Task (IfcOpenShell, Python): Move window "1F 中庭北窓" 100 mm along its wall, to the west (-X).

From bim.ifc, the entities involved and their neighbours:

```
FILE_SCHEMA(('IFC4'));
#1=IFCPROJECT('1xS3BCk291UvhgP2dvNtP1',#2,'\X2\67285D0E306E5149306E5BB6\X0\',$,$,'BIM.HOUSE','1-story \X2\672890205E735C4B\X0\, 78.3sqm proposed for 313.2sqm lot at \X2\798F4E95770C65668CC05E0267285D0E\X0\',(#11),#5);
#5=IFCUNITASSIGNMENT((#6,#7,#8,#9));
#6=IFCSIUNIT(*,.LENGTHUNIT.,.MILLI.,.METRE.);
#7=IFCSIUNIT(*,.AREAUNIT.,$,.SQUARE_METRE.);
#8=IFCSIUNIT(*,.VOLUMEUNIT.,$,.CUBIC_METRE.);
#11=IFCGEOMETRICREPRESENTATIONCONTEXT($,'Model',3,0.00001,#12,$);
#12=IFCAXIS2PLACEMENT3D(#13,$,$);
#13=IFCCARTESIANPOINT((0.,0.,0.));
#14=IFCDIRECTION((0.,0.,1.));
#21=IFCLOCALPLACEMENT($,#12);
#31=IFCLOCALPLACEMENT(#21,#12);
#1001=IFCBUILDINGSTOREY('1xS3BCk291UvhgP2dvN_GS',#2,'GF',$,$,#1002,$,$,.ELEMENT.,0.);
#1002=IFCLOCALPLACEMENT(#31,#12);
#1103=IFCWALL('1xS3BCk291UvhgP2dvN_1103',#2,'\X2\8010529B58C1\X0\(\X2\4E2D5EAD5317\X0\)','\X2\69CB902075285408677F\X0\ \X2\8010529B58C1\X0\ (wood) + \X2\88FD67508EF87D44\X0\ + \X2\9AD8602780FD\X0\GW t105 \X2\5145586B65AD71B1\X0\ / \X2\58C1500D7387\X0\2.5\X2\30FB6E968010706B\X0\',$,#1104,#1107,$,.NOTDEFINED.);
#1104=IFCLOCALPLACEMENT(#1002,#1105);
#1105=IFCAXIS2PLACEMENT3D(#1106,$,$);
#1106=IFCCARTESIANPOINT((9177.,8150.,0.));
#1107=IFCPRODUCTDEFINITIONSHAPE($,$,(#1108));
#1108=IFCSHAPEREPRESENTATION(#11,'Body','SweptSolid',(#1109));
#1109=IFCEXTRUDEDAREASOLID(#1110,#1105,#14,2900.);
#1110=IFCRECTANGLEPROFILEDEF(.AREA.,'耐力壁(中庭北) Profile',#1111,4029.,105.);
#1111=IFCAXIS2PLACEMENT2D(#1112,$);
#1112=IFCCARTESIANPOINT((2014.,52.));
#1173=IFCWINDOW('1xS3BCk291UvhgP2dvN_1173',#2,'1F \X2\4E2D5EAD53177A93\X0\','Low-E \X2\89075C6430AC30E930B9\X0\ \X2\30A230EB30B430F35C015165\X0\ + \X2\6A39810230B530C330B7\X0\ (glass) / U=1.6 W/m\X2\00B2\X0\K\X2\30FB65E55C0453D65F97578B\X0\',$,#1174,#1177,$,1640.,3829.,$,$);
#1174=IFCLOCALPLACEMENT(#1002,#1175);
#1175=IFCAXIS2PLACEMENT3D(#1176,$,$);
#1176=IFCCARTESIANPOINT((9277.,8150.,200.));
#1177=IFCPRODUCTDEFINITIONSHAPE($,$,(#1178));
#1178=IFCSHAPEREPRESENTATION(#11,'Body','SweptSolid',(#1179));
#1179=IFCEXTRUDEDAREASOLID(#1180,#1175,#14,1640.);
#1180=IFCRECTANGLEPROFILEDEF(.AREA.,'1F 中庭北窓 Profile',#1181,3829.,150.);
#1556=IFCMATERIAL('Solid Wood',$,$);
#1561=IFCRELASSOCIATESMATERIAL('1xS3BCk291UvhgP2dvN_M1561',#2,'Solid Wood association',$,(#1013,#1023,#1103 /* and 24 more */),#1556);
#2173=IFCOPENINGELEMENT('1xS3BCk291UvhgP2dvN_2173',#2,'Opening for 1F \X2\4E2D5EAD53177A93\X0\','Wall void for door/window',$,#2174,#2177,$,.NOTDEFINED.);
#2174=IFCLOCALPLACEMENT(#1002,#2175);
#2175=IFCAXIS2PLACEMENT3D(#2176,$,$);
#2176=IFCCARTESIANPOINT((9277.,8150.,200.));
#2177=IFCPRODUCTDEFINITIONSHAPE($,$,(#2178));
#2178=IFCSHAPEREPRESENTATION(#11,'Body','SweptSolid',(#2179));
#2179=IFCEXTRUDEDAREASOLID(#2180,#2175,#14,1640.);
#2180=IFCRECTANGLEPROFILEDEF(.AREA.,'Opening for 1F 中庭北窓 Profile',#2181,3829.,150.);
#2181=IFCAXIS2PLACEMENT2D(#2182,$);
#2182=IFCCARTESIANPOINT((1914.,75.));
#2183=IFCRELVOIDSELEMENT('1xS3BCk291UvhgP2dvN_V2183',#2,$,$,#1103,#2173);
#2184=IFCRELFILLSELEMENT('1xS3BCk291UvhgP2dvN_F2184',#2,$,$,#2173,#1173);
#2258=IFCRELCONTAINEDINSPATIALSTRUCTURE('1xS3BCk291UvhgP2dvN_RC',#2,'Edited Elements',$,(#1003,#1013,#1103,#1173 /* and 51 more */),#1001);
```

```python
import ifcopenshell
import ifcopenshell.api.geometry
import ifcopenshell.util.placement
import ifcopenshell.util.unit

model = ifcopenshell.open("bim.ifc")
unit_scale = ifcopenshell.util.unit.calculate_unit_scale(model)

window = model.by_guid("1xS3BCk291UvhgP2dvN_1173")
opening = window.FillsVoids[0].RelatingOpeningElement
wall = opening.VoidsElements[0].RelatingBuildingElement

wall_matrix = ifcopenshell.util.placement.get_local_placement(wall.ObjectPlacement)
shift = wall_matrix[:3, 0] * -0.1 / unit_scale
before = ifcopenshell.util.placement.get_local_placement(window.ObjectPlacement)[:3, 3].copy()

# The window is not placed relative to its opening, so move both.
for product in (opening, window):
    matrix = ifcopenshell.util.placement.get_local_placement(product.ObjectPlacement)
    matrix[:3, 3] += shift
    ifcopenshell.api.geometry.edit_object_placement(model, product=product, matrix=matrix, is_si=False)

after = ifcopenshell.util.placement.get_local_placement(window.ObjectPlacement)[:3, 3]
print("window moved by", (after - before).round(3) + 0.0)

model.write("bim_updated.ifc")
```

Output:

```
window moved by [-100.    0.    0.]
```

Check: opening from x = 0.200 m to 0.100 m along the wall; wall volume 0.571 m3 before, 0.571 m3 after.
